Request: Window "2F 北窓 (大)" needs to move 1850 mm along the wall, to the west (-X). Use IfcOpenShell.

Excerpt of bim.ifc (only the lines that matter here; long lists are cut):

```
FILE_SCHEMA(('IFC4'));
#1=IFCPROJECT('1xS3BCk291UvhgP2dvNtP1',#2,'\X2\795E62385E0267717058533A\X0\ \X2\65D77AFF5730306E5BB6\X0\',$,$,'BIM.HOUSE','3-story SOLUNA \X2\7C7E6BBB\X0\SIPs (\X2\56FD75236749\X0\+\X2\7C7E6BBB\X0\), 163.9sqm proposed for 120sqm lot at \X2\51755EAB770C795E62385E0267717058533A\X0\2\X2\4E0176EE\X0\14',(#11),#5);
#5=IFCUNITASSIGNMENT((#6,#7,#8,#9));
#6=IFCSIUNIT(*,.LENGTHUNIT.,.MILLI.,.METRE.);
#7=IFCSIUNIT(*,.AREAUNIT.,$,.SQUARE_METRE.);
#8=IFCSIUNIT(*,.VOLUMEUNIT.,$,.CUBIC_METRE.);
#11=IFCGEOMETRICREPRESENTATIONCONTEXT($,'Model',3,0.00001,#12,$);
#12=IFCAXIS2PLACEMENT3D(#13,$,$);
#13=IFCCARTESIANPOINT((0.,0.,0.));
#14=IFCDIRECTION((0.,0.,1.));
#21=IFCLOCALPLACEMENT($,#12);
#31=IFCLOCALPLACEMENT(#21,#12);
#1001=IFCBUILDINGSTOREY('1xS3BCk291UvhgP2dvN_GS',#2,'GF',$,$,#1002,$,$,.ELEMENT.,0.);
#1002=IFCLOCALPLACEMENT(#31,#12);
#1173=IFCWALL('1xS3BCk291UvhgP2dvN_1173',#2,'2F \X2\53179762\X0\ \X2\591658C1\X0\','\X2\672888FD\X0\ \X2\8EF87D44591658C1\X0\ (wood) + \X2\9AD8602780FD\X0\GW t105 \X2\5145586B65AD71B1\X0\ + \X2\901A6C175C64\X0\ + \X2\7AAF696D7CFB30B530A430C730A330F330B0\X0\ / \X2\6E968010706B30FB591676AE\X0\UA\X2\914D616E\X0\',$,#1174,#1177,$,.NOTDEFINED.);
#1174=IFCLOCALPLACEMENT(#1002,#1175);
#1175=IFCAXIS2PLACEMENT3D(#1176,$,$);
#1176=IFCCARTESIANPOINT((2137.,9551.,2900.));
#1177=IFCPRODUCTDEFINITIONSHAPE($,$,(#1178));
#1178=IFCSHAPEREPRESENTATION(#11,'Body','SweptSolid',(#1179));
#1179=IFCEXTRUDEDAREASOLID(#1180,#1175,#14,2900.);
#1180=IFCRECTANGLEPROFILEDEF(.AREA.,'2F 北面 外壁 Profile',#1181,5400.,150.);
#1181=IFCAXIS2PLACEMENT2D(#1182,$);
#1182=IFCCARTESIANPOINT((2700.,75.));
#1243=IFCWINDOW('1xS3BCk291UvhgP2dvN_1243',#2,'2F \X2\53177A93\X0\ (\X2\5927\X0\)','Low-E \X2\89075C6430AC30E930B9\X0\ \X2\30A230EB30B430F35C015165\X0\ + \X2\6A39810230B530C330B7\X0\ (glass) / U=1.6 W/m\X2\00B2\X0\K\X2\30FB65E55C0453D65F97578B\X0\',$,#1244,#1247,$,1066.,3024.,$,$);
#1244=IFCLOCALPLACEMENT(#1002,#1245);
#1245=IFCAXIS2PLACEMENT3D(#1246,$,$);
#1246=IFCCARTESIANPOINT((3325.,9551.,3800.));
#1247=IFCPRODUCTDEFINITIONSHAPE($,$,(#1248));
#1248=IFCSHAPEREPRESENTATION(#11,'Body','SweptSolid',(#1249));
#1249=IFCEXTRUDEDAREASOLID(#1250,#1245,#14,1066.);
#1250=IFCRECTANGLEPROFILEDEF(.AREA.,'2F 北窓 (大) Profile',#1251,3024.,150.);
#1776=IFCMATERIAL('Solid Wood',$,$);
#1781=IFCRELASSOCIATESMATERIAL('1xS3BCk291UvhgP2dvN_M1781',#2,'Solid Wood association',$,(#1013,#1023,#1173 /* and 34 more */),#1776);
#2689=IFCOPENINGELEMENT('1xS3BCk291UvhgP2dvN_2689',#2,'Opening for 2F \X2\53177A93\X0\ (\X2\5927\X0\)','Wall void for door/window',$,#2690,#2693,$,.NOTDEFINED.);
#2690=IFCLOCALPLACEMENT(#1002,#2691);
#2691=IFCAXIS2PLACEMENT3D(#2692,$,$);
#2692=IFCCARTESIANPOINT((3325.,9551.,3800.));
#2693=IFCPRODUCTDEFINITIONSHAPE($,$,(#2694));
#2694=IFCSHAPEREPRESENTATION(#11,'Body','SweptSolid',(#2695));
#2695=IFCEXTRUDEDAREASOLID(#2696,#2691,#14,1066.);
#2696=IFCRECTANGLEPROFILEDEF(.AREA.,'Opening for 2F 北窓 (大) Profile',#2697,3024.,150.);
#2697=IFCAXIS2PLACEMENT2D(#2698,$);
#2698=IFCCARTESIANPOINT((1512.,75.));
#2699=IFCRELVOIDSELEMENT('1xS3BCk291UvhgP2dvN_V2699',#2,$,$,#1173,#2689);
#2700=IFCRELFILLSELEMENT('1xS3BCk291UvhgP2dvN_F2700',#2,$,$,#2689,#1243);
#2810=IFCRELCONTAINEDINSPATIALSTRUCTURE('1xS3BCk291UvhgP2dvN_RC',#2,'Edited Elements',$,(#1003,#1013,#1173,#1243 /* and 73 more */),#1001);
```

```python
import ifcopenshell
import ifcopenshell.api.geometry
import ifcopenshell.util.placement
import ifcopenshell.util.unit

model = ifcopenshell.open("bim.ifc")
unit_scale = ifcopenshell.util.unit.calculate_unit_scale(model)

window = model.by_guid("1xS3BCk291UvhgP2dvN_1243")
opening = window.FillsVoids[0].RelatingOpeningElement
wall = opening.VoidsElements[0].RelatingBuildingElement

wall_matrix = ifcopenshell.util.placement.get_local_placement(wall.ObjectPlacement)
shift = wall_matrix[:3, 0] * -1.85 / unit_scale
before = ifcopenshell.util.placement.get_local_placement(window.ObjectPlacement)[:3, 3].copy()

# The window is not placed relative to its opening, so move both.
for product in (opening, window):
    matrix = ifcopenshell.util.placement.get_local_placement(product.ObjectPlacement)
    matrix[:3, 3] += shift
    ifcopenshell.api.geometry.edit_object_placement(model, product=product, matrix=matrix, is_si=False)

after = ifcopenshell.util.placement.get_local_placement(window.ObjectPlacement)[:3, 3]
print("window moved by", (after - before).round(3) + 0.0)

model.write("bim_updated.ifc")
```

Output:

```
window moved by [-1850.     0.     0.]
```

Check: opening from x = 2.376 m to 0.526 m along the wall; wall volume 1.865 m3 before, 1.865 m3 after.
